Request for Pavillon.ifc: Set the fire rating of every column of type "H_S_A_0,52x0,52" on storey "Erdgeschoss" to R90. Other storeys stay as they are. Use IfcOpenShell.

First a look at what the model holds.

```python
import ifcopenshell
import ifcopenshell.util.element

model = ifcopenshell.open("Pavillon.ifc")
print(model.schema)
storey = next(s for s in model.by_type("IfcBuildingStorey") if s.Name == "Erdgeschoss")
columns = [e for e in ifcopenshell.util.element.get_decomposition(storey) if e.is_a("IfcColumn")]
seen = {}
for e in columns:
    element_type = ifcopenshell.util.element.get_type(e)
    key = (element_type.Name if element_type != e and element_type else None, ifcopenshell.util.element.get_pset(e, "Pset_ColumnCommon", "FireRating"))
    seen[key] = seen.get(key, 0) + 1
for (name, value), count in sorted(seen.items(), key=str):
    print(count, "x", name, "|", value)
```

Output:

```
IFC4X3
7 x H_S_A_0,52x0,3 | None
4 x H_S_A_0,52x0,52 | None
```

```python
import ifcopenshell
import ifcopenshell.api.pset
import ifcopenshell.util.element

model = ifcopenshell.open("Pavillon.ifc")

storey = next(s for s in model.by_type("IfcBuildingStorey") if s.Name == "Erdgeschoss")
columns = [e for e in ifcopenshell.util.element.get_decomposition(storey) if e.is_a("IfcColumn")]

count = 0
for e in columns:
    element_type = ifcopenshell.util.element.get_type(e)
    if element_type in (None, e) or element_type.Name != "H_S_A_0,52x0,52":
        continue
    # add_pset returns the element's existing set when there is one.
    pset = ifcopenshell.api.pset.add_pset(model, product=e, name="Pset_ColumnCommon")
    ifcopenshell.api.pset.edit_pset(model, pset=pset, properties={"FireRating": "R90"})
    count += 1

print(count, "columns updated")

model.write("Pavillon_edited.ifc")
```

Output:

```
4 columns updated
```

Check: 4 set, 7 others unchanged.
